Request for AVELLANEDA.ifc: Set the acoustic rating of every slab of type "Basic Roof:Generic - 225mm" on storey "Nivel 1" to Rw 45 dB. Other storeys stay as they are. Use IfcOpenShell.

First a look at what the model holds.

```python
import ifcopenshell
import ifcopenshell.util.element

model = ifcopenshell.open("AVELLANEDA.ifc")
print(model.schema)
storey = next(s for s in model.by_type("IfcBuildingStorey") if s.Name == "Nivel 1")
slabs = [e for e in ifcopenshell.util.element.get_decomposition(storey) if e.is_a("IfcSlab")]
seen = {}
for e in slabs:
    element_type = ifcopenshell.util.element.get_type(e)
    key = (element_type.Name if element_type != e and element_type else None, ifcopenshell.util.element.get_pset(e, "Pset_SlabCommon", "AcousticRating"))
    seen[key] = seen.get(key, 0) + 1
for (name, value), count in sorted(seen.items(), key=str):
    print(count, "x", name, "|", value)
```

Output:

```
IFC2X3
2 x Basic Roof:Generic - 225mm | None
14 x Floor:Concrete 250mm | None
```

```python
import ifcopenshell
import ifcopenshell.api.pset
import ifcopenshell.util.element

model = ifcopenshell.open("AVELLANEDA.ifc")

storey = next(s for s in model.by_type("IfcBuildingStorey") if s.Name == "Nivel 1")
slabs = [e for e in ifcopenshell.util.element.get_decomposition(storey) if e.is_a("IfcSlab")]

count = 0
for e in slabs:
    element_type = ifcopenshell.util.element.get_type(e)
    if element_type in (None, e) or element_type.Name != "Basic Roof:Generic - 225mm":
        continue
    # add_pset returns the element's existing set when there is one.
    pset = ifcopenshell.api.pset.add_pset(model, product=e, name="Pset_SlabCommon")
    ifcopenshell.api.pset.edit_pset(model, pset=pset, properties={"AcousticRating": "Rw 45 dB"})
    count += 1

print(count, "slabs updated")

model.write("AVELLANEDA_edited.ifc")
```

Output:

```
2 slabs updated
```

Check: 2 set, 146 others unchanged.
